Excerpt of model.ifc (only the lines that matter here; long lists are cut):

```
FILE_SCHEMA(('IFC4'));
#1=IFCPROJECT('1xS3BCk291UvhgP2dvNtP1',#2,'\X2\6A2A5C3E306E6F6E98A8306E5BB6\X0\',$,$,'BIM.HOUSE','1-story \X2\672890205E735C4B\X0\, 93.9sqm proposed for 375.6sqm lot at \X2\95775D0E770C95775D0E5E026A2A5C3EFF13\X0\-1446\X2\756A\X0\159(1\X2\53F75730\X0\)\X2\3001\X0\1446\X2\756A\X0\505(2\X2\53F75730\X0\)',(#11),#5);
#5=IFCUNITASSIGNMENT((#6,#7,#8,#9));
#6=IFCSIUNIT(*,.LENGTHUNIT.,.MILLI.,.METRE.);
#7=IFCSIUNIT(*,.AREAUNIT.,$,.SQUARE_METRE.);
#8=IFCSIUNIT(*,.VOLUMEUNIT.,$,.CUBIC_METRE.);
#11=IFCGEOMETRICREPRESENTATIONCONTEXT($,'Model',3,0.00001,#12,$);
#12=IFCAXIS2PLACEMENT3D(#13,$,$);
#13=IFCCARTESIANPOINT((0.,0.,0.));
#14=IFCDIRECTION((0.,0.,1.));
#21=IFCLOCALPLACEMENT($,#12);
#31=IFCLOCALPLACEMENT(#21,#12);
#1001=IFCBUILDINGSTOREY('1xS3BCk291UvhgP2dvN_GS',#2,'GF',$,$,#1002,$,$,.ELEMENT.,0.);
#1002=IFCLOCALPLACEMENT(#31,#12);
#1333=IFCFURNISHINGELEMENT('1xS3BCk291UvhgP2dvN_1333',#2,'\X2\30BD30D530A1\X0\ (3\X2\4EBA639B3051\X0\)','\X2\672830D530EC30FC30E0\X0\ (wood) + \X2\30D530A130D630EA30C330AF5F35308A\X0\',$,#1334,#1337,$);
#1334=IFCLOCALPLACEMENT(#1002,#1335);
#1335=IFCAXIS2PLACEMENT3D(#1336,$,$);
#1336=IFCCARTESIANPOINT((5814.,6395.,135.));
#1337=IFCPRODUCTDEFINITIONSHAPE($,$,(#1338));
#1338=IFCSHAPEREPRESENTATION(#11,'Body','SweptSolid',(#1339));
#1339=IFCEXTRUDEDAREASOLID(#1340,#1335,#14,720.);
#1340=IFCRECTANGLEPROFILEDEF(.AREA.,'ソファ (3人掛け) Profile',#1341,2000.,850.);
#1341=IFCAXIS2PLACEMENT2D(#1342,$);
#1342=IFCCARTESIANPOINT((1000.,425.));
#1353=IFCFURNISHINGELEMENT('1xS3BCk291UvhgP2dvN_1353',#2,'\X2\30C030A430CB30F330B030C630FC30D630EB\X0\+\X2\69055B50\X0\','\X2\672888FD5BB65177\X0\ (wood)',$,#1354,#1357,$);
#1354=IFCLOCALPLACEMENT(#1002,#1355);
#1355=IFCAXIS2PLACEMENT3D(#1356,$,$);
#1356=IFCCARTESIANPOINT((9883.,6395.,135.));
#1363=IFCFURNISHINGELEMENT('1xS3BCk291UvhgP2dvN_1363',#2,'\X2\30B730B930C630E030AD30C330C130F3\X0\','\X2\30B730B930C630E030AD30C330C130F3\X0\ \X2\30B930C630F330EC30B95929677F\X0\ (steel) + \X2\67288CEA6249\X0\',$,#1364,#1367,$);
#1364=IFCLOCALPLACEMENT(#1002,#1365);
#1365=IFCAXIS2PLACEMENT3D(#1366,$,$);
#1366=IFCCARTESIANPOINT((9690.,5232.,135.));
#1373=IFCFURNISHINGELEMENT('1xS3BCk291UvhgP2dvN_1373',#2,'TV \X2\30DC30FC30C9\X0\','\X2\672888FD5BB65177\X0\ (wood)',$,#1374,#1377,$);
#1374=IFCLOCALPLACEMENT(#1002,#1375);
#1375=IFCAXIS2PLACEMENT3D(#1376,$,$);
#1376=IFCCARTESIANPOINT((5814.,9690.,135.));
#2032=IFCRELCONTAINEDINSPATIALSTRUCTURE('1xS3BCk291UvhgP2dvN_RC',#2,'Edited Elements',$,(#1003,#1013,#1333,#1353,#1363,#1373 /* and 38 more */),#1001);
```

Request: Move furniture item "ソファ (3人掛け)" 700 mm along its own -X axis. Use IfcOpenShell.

```python
import ifcopenshell
import ifcopenshell.api.geometry
import ifcopenshell.util.placement
import ifcopenshell.util.unit

model = ifcopenshell.open("model.ifc")
unit_scale = ifcopenshell.util.unit.calculate_unit_scale(model)

item = model.by_id(1333)
matrix = ifcopenshell.util.placement.get_local_placement(item.ObjectPlacement)
matrix[:3, 3] -= matrix[:3, 0] * 0.7 / unit_scale
ifcopenshell.api.geometry.edit_object_placement(model, product=item, matrix=matrix, is_si=False)

print(ifcopenshell.util.placement.get_local_placement(item.ObjectPlacement).round(3) + 0.0)

model.write("model-out.ifc")
```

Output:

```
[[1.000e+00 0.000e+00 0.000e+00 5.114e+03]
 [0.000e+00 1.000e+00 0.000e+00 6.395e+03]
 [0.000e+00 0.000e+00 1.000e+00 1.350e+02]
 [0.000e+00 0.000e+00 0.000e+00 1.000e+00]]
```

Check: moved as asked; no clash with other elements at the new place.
